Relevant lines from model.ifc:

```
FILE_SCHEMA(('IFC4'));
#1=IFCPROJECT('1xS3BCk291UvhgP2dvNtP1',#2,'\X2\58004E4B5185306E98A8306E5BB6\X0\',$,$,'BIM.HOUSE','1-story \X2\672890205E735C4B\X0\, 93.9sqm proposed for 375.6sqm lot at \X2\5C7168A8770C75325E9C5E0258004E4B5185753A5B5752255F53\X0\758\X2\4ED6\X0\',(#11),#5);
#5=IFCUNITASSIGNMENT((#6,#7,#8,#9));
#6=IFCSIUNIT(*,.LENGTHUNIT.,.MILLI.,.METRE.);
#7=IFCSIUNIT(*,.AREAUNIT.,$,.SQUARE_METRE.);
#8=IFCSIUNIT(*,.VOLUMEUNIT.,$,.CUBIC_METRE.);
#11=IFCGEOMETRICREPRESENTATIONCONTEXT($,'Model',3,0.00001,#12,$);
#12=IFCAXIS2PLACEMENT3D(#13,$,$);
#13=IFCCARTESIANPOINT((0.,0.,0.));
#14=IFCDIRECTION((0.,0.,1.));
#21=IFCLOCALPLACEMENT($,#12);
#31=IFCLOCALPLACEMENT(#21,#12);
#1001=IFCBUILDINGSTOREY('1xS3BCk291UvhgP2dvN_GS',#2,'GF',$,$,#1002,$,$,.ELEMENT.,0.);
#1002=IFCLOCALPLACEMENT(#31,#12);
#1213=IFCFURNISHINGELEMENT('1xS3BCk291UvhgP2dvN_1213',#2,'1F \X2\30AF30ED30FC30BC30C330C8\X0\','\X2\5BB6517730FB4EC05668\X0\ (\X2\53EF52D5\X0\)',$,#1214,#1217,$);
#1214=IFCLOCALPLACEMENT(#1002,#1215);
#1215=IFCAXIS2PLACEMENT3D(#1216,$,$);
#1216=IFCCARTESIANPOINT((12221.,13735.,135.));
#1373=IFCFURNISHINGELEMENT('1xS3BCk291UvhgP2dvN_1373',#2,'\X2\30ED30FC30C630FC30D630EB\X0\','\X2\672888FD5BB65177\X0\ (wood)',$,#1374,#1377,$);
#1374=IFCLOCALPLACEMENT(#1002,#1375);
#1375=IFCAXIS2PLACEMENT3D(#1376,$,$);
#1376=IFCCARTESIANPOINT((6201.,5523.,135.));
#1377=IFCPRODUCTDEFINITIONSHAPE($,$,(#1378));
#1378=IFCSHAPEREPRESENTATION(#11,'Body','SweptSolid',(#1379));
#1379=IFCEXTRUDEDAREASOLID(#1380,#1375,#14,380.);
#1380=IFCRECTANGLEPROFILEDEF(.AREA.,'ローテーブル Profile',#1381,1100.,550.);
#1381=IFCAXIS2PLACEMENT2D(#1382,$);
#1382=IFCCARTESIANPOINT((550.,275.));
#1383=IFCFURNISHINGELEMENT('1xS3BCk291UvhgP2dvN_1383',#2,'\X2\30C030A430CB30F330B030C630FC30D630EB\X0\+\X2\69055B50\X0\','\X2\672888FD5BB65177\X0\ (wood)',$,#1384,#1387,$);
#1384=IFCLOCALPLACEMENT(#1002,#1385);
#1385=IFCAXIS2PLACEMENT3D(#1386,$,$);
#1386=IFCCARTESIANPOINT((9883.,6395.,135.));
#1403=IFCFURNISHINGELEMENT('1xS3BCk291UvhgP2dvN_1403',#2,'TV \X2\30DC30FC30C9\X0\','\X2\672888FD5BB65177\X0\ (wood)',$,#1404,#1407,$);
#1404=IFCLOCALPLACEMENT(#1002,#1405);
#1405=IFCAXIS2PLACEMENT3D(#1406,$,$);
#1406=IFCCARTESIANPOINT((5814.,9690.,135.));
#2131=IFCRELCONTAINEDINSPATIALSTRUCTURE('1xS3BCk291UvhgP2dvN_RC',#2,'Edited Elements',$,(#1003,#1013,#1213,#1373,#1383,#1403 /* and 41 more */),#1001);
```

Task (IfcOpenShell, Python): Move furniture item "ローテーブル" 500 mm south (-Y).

```python
import ifcopenshell
import ifcopenshell.api.geometry
import ifcopenshell.util.placement
import ifcopenshell.util.unit

model = ifcopenshell.open("model.ifc")
unit_scale = ifcopenshell.util.unit.calculate_unit_scale(model)

item = model.by_id(1373)
matrix = ifcopenshell.util.placement.get_local_placement(item.ObjectPlacement)
matrix[1, 3] -= 0.5 / unit_scale
ifcopenshell.api.geometry.edit_object_placement(model, product=item, matrix=matrix, is_si=False)

print(ifcopenshell.util.placement.get_local_placement(item.ObjectPlacement).round(3) + 0.0)

model.write("model-out.ifc")
```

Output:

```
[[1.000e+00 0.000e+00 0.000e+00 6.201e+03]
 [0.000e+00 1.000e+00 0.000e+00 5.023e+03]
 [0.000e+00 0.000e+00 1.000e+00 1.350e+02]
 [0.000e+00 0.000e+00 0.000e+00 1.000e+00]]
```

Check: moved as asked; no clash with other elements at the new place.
